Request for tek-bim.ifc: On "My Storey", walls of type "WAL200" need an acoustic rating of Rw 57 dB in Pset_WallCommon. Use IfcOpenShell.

First a look at what the model holds.

```python
import ifcopenshell
import ifcopenshell.util.element

model = ifcopenshell.open("tek-bim.ifc")
print(model.schema)
storey = next(s for s in model.by_type("IfcBuildingStorey") if s.Name == "My Storey")
walls = [e for e in ifcopenshell.util.element.get_decomposition(storey) if e.is_a("IfcWall")]
seen = {}
for e in walls:
    element_type = ifcopenshell.util.element.get_type(e)
    key = (element_type.Name if element_type != e and element_type else None, ifcopenshell.util.element.get_pset(e, "Pset_WallCommon", "AcousticRating"))
    seen[key] = seen.get(key, 0) + 1
for (name, value), count in sorted(seen.items(), key=str):
    print(count, "x", name, "|", value)
```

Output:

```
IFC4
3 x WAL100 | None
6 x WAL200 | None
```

```python
import ifcopenshell
import ifcopenshell.api.pset
import ifcopenshell.util.element

model = ifcopenshell.open("tek-bim.ifc")

storey = next(s for s in model.by_type("IfcBuildingStorey") if s.Name == "My Storey")
walls = [e for e in ifcopenshell.util.element.get_decomposition(storey) if e.is_a("IfcWall")]

count = 0
for e in walls:
    element_type = ifcopenshell.util.element.get_type(e)
    if element_type in (None, e) or element_type.Name != "WAL200":
        continue
    # add_pset returns the element's existing set when there is one.
    pset = ifcopenshell.api.pset.add_pset(model, product=e, name="Pset_WallCommon")
    ifcopenshell.api.pset.edit_pset(model, pset=pset, properties={"AcousticRating": "Rw 57 dB"})
    count += 1

print(count, "walls updated")

model.write("tek-bim_updated.ifc")
```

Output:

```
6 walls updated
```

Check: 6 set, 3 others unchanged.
